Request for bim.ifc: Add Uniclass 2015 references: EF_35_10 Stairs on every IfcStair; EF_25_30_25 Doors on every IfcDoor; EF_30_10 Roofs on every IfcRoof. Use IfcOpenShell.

First a look at what the model holds.

```python
import ifcopenshell

model = ifcopenshell.open("bim.ifc")
print(model.schema)
print("classifications:", [c.Name for c in model.by_type("IfcClassification")])
for ifc_class in ("IfcDoor", "IfcRoof", "IfcStair", "IfcWall", "IfcWindow"):
    print(ifc_class, len(model.by_type(ifc_class)))
```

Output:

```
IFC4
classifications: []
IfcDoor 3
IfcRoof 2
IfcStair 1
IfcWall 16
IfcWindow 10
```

```python
import ifcopenshell
import ifcopenshell.api.classification

model = ifcopenshell.open("bim.ifc")

system = ifcopenshell.api.classification.add_classification(model, classification="Uniclass 2015")

codes = {
    "IfcStair": ("EF_35_10", "Stairs"),
    "IfcDoor": ("EF_25_30_25", "Doors"),
    "IfcRoof": ("EF_30_10", "Roofs"),
}
for ifc_class, (code, name) in codes.items():
    products = model.by_type(ifc_class)
    ifcopenshell.api.classification.add_reference(
        model, products=products, classification=system, identification=code, name=name
    )
    print(code, len(products))

model.write("bim_edited.ifc")
```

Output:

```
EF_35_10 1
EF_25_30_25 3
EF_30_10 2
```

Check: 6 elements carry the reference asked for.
